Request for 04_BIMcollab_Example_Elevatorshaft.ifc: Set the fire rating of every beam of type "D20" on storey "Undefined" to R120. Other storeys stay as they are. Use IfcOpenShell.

First a look at what the model holds.

```python
import ifcopenshell
import ifcopenshell.util.element

model = ifcopenshell.open("04_BIMcollab_Example_Elevatorshaft.ifc")
print(model.schema)
storey = next(s for s in model.by_type("IfcBuildingStorey") if s.Name == "Undefined")
beams = [e for e in ifcopenshell.util.element.get_decomposition(storey) if e.is_a("IfcBeam")]
seen = {}
for e in beams:
    element_type = ifcopenshell.util.element.get_type(e)
    key = (element_type.Name if element_type != e and element_type else None, ifcopenshell.util.element.get_pset(e, "Pset_BeamCommon", "FireRating"))
    seen[key] = seen.get(key, 0) + 1
for (name, value), count in sorted(seen.items(), key=str):
    print(count, "x", name, "|", value)
```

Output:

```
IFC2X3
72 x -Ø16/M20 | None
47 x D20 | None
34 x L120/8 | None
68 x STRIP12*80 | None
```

```python
import ifcopenshell
import ifcopenshell.api.pset
import ifcopenshell.util.element

model = ifcopenshell.open("04_BIMcollab_Example_Elevatorshaft.ifc")

storey = next(s for s in model.by_type("IfcBuildingStorey") if s.Name == "Undefined")
beams = [e for e in ifcopenshell.util.element.get_decomposition(storey) if e.is_a("IfcBeam")]

count = 0
for e in beams:
    element_type = ifcopenshell.util.element.get_type(e)
    if element_type in (None, e) or element_type.Name != "D20":
        continue
    # add_pset returns the element's existing set when there is one.
    pset = ifcopenshell.api.pset.add_pset(model, product=e, name="Pset_BeamCommon")
    ifcopenshell.api.pset.edit_pset(model, pset=pset, properties={"FireRating": "R120"})
    count += 1

print(count, "beams updated")

model.write("04_BIMcollab_Example_Elevatorshaft_edited.ifc")
```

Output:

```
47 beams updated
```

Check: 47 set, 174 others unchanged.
